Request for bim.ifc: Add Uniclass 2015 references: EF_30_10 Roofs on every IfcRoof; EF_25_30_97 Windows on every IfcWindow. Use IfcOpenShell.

First a look at what the model holds.

```python
import ifcopenshell

model = ifcopenshell.open("bim.ifc")
print(model.schema)
print("classifications:", [c.Name for c in model.by_type("IfcClassification")])
for ifc_class in ("IfcDoor", "IfcRoof", "IfcStair", "IfcWall", "IfcWindow"):
    print(ifc_class, len(model.by_type(ifc_class)))
```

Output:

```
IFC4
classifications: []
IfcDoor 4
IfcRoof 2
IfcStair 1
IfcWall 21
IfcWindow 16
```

```python
import ifcopenshell
import ifcopenshell.api.classification

model = ifcopenshell.open("bim.ifc")

system = ifcopenshell.api.classification.add_classification(model, classification="Uniclass 2015")

codes = {
    "IfcRoof": ("EF_30_10", "Roofs"),
    "IfcWindow": ("EF_25_30_97", "Windows"),
}
for ifc_class, (code, name) in codes.items():
    products = model.by_type(ifc_class)
    ifcopenshell.api.classification.add_reference(
        model, products=products, classification=system, identification=code, name=name
    )
    print(code, len(products))

model.write("bim-out.ifc")
```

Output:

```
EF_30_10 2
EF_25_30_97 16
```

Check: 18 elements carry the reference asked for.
